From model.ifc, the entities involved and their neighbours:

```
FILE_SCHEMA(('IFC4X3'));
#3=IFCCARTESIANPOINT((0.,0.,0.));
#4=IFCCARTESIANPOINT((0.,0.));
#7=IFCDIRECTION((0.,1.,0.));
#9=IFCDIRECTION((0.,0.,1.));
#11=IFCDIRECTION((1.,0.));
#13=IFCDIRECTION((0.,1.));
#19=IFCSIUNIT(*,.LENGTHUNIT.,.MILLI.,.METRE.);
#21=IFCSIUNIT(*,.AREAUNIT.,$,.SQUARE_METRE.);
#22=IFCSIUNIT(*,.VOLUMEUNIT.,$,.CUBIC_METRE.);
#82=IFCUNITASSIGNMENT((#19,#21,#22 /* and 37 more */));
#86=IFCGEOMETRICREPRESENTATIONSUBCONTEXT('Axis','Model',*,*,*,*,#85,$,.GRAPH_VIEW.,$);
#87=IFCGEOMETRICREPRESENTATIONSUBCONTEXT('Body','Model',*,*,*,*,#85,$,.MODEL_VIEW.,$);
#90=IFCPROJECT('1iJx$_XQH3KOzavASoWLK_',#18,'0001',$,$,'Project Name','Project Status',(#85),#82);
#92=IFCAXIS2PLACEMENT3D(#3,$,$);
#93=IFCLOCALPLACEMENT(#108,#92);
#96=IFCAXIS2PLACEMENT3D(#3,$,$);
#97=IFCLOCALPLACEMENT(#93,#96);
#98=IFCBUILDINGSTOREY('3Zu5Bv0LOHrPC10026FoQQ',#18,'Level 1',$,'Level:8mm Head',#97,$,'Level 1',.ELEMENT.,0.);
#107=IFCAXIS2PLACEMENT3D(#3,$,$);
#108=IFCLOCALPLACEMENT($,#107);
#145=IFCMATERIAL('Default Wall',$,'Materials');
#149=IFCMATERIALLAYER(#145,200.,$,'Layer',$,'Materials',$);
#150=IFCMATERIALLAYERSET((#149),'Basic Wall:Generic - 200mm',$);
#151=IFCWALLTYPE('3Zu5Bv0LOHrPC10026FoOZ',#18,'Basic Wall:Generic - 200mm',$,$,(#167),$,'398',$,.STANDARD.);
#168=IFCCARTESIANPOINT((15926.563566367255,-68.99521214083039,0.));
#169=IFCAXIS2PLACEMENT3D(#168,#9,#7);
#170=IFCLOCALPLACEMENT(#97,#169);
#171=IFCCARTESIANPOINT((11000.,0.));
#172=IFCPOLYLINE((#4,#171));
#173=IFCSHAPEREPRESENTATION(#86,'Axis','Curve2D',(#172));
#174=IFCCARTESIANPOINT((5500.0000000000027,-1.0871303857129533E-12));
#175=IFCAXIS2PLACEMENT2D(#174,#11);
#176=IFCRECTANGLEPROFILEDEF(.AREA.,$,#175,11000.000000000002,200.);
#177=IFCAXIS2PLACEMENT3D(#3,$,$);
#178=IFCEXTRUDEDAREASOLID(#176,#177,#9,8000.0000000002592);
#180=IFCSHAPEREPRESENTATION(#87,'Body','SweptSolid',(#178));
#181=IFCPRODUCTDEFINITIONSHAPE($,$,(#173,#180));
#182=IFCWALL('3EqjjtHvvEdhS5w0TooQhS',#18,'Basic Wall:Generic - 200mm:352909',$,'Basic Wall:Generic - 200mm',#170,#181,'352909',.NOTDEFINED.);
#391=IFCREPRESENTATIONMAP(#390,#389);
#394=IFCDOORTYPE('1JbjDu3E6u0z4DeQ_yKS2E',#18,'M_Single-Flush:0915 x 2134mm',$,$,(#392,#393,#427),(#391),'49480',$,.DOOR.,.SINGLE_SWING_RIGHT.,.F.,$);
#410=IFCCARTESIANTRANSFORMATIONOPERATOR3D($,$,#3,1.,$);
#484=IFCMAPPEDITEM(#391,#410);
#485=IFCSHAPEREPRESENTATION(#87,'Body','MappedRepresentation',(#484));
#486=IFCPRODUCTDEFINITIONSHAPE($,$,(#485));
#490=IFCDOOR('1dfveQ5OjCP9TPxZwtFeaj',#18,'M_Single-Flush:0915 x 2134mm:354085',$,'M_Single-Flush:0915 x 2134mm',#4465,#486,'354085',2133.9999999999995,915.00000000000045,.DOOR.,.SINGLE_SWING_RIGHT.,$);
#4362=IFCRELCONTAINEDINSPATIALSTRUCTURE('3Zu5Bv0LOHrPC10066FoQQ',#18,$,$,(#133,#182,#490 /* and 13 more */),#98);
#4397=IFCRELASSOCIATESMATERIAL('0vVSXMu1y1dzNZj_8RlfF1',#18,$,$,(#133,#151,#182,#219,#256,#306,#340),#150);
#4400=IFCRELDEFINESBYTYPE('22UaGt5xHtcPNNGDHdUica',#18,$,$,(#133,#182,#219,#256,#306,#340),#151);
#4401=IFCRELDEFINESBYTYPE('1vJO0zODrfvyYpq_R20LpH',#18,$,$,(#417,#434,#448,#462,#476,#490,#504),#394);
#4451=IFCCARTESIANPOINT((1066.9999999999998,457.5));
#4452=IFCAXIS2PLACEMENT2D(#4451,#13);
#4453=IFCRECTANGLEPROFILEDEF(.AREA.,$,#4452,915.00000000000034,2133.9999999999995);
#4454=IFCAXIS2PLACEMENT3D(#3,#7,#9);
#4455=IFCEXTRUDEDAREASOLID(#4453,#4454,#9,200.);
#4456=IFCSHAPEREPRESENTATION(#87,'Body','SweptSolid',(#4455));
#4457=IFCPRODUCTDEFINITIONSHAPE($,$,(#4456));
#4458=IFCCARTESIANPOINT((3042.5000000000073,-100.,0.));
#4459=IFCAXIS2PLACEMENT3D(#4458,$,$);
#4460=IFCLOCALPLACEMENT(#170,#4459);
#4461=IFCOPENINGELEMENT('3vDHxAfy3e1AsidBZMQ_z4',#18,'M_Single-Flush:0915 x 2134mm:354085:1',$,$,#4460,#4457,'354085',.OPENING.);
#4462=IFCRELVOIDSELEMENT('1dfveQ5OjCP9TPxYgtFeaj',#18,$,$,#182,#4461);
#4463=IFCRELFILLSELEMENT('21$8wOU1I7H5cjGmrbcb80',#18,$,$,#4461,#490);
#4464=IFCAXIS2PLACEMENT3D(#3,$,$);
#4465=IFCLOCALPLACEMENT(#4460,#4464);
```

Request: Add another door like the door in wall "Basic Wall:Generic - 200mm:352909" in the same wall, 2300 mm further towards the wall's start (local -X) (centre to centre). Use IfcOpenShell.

```python
import ifcopenshell
import ifcopenshell.api.feature
import ifcopenshell.api.geometry
import ifcopenshell.api.root
import ifcopenshell.geom
import ifcopenshell.util.element
import ifcopenshell.util.placement
import ifcopenshell.util.shape

model = ifcopenshell.open("model.ifc")
settings = ifcopenshell.geom.settings()


def volume(element):
    """Net volume in cubic metres, openings subtracted."""
    shape = ifcopenshell.geom.create_shape(settings, element)
    return ifcopenshell.util.shape.get_volume(shape.geometry)


def reuse_history(source, copy):
    """copy_class also copies each property set's owner history, people and application; keep the originals."""
    for rel in copy.IsDefinedBy:
        if rel.is_a("IfcRelDefinesByProperties") and (history := rel.RelatingPropertyDefinition.OwnerHistory):
            rel.RelatingPropertyDefinition.OwnerHistory = source.OwnerHistory
            ifcopenshell.util.element.remove_deep2(model, history)


door = model.by_id(490)
opening = door.FillsVoids[0].RelatingOpeningElement
wall = opening.VoidsElements[0].RelatingBuildingElement
before = volume(wall)
shift = ifcopenshell.util.placement.get_local_placement(wall.ObjectPlacement)[:3, 0] * -2300.0

# copy_class copies the void relationship, type, container and properties, but no geometry.
new_opening = ifcopenshell.api.root.copy_class(model, product=opening)
new_opening.Representation = ifcopenshell.util.element.copy_deep(
    model, opening.Representation, exclude=["IfcGeometricRepresentationContext", "IfcRepresentationMap"]
)
new_opening.Name = "M_Single-Flush:0915 x 2134mm"
new_opening.Tag = None
new_door = ifcopenshell.api.root.copy_class(model, product=door)
new_door.Representation = ifcopenshell.util.element.copy_deep(
    model, door.Representation, exclude=["IfcGeometricRepresentationContext", "IfcRepresentationMap"]
)
new_door.Name = "M_Single-Flush:0915 x 2134mm"
new_door.Tag = None
reuse_history(door, new_door)
ifcopenshell.api.feature.add_filling(model, opening=new_opening, element=new_door)

for old, new in ((opening, new_opening), (door, new_door)):
    matrix = ifcopenshell.util.placement.get_local_placement(old.ObjectPlacement)
    matrix[:3, 3] += shift
    ifcopenshell.api.geometry.edit_object_placement(model, product=new, matrix=matrix, is_si=False)

after = volume(wall)

print(f"wall volume {before:.3f} -> {after:.3f} m3")

model.write("model-out.ifc")
```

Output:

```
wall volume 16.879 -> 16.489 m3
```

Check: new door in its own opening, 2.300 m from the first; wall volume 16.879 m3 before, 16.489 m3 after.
